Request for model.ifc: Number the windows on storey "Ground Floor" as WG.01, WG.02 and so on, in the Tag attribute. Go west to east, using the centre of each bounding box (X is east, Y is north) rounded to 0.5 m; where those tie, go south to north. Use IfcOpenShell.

First a look at what the model holds.

```python
import ifcopenshell
import ifcopenshell.util.element
import ifcopenshell.util.placement

model = ifcopenshell.open("model.ifc")
print(model.schema)
storey = next(s for s in model.by_type("IfcBuildingStorey") if s.Name == "Ground Floor")
windows = [e for e in ifcopenshell.util.element.get_decomposition(storey) if e.is_a("IfcWindow")]
for e in sorted(windows, key=lambda e: e.id()):
    origin = ifcopenshell.util.placement.get_local_placement(e.ObjectPlacement)[:3, 3]
    print(e.id(), e.Tag, e.Name, origin.round(2) + 0.0, sep=" | ")
```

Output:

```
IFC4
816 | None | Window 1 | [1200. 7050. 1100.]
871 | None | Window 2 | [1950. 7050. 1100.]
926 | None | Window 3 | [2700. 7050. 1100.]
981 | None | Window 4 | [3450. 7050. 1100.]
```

```python
import ifcopenshell
import ifcopenshell.geom
import ifcopenshell.util.element
import ifcopenshell.util.shape

model = ifcopenshell.open("model.ifc")
settings = ifcopenshell.geom.settings()
settings.set("use-world-coords", True)


def centre(element):
    shape = ifcopenshell.geom.create_shape(settings, element)
    return ifcopenshell.util.shape.get_bbox_centroid(shape.geometry)


storey = next(s for s in model.by_type("IfcBuildingStorey") if s.Name == "Ground Floor")
windows = [e for e in ifcopenshell.util.element.get_decomposition(storey) if e.is_a("IfcWindow")]

# Insertion points can sit at a corner or the storey origin, so sort by the geometry (in metres).
centres = {e: centre(e) for e in windows}
windows.sort(key=lambda e: (round(centres[e][0] / 0.5), centres[e][1]))

for i, e in enumerate(windows, start=1):
    number = f"WG.{i:02d}"
    e.Tag = number
    print(e.id(), number)

model.write("model_rev.ifc")
```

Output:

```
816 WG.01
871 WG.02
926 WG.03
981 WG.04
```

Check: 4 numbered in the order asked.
